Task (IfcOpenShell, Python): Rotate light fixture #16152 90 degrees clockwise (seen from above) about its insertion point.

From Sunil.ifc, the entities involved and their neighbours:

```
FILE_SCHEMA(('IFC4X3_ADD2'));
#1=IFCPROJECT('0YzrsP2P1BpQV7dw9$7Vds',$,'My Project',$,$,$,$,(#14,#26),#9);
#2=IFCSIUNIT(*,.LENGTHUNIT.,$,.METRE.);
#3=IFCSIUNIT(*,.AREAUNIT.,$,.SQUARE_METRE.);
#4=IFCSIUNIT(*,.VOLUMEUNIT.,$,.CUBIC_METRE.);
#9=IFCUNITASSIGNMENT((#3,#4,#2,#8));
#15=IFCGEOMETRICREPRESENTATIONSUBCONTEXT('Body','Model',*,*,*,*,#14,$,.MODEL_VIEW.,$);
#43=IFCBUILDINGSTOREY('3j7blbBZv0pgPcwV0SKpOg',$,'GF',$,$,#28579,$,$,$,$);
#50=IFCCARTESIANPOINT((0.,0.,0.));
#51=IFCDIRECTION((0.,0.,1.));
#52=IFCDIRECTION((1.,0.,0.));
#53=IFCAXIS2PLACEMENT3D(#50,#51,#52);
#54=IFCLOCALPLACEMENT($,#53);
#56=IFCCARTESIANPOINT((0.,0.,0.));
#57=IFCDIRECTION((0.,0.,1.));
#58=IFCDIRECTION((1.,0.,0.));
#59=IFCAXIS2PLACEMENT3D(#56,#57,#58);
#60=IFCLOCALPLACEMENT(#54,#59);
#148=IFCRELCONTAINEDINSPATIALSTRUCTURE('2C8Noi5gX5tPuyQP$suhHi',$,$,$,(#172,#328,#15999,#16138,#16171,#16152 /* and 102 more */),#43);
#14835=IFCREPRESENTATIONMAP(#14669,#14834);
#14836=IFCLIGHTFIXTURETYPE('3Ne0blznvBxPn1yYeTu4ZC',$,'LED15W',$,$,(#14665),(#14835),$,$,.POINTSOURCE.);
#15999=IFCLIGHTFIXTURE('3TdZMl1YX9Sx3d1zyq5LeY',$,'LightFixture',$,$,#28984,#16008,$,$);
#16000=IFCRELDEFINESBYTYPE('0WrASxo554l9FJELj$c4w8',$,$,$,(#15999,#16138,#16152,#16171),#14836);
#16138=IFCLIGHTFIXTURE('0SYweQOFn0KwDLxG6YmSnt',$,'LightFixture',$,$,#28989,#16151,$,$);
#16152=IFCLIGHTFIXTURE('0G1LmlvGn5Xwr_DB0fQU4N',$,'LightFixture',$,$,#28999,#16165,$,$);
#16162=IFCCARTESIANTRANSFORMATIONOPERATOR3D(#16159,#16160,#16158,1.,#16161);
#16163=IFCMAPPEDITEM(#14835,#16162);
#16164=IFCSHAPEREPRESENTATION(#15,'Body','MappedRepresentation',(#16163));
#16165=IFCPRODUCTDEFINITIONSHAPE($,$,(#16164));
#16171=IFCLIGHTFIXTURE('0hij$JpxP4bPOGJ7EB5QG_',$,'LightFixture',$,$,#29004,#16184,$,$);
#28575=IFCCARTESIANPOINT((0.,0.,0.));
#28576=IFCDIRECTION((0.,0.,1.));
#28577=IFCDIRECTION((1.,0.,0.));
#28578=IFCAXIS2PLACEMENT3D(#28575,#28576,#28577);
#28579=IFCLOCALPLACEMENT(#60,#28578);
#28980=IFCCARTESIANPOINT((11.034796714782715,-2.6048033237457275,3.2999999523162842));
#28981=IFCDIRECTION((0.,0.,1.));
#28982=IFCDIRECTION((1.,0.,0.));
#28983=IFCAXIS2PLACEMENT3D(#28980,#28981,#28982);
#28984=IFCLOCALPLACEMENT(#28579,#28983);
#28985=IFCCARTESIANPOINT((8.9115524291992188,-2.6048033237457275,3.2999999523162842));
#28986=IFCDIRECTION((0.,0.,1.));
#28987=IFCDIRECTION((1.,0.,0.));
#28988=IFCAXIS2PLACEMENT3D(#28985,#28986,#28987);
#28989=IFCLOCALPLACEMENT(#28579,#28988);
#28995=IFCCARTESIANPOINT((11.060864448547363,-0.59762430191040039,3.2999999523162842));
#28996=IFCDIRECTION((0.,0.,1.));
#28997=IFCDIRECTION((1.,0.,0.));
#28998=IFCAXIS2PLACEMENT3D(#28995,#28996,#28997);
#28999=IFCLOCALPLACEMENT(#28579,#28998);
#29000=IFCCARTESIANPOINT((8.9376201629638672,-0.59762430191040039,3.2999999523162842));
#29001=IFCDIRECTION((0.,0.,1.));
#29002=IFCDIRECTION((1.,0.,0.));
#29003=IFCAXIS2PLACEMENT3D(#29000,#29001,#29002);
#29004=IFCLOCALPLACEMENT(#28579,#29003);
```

```python
import ifcopenshell
import ifcopenshell.api.geometry
import ifcopenshell.util.placement

model = ifcopenshell.open("Sunil.ifc")

item = model.by_guid("0G1LmlvGn5Xwr_DB0fQU4N")
matrix = ifcopenshell.util.placement.get_local_placement(item.ObjectPlacement)
matrix = matrix @ ifcopenshell.util.placement.rotation(-90, "Z")
ifcopenshell.api.geometry.edit_object_placement(model, product=item, matrix=matrix, is_si=False)

print(ifcopenshell.util.placement.get_local_placement(item.ObjectPlacement).round(3) + 0.0)

model.write("Sunil_v2.ifc")
```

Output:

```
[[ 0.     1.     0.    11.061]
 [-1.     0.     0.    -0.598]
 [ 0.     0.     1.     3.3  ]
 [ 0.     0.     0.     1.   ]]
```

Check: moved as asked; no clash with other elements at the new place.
